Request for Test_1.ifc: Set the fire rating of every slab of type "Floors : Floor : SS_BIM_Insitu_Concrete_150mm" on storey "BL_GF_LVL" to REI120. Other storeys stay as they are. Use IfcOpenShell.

First a look at what the model holds.

```python
import ifcopenshell
import ifcopenshell.util.element

model = ifcopenshell.open("Test_1.ifc")
print(model.schema)
storey = next(s for s in model.by_type("IfcBuildingStorey") if s.Name == "BL_GF_LVL")
slabs = [e for e in ifcopenshell.util.element.get_decomposition(storey) if e.is_a("IfcSlab")]
seen = {}
for e in slabs:
    element_type = ifcopenshell.util.element.get_type(e)
    key = (element_type.Name if element_type != e and element_type else None, ifcopenshell.util.element.get_pset(e, "Pset_SlabCommon", "FireRating"))
    seen[key] = seen.get(key, 0) + 1
for (name, value), count in sorted(seen.items(), key=str):
    print(count, "x", name, "|", value)
```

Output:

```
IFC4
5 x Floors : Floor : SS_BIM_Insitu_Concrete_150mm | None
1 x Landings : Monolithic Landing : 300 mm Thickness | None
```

```python
import ifcopenshell
import ifcopenshell.api.pset
import ifcopenshell.util.element

model = ifcopenshell.open("Test_1.ifc")

storey = next(s for s in model.by_type("IfcBuildingStorey") if s.Name == "BL_GF_LVL")
slabs = [e for e in ifcopenshell.util.element.get_decomposition(storey) if e.is_a("IfcSlab")]

count = 0
for e in slabs:
    element_type = ifcopenshell.util.element.get_type(e)
    if element_type in (None, e) or element_type.Name != "Floors : Floor : SS_BIM_Insitu_Concrete_150mm":
        continue
    # add_pset returns the element's existing set when there is one.
    pset = ifcopenshell.api.pset.add_pset(model, product=e, name="Pset_SlabCommon")
    ifcopenshell.api.pset.edit_pset(model, pset=pset, properties={"FireRating": "REI120"})
    count += 1

print(count, "slabs updated")

model.write("Test_1_rev.ifc")
```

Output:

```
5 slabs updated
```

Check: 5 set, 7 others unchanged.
